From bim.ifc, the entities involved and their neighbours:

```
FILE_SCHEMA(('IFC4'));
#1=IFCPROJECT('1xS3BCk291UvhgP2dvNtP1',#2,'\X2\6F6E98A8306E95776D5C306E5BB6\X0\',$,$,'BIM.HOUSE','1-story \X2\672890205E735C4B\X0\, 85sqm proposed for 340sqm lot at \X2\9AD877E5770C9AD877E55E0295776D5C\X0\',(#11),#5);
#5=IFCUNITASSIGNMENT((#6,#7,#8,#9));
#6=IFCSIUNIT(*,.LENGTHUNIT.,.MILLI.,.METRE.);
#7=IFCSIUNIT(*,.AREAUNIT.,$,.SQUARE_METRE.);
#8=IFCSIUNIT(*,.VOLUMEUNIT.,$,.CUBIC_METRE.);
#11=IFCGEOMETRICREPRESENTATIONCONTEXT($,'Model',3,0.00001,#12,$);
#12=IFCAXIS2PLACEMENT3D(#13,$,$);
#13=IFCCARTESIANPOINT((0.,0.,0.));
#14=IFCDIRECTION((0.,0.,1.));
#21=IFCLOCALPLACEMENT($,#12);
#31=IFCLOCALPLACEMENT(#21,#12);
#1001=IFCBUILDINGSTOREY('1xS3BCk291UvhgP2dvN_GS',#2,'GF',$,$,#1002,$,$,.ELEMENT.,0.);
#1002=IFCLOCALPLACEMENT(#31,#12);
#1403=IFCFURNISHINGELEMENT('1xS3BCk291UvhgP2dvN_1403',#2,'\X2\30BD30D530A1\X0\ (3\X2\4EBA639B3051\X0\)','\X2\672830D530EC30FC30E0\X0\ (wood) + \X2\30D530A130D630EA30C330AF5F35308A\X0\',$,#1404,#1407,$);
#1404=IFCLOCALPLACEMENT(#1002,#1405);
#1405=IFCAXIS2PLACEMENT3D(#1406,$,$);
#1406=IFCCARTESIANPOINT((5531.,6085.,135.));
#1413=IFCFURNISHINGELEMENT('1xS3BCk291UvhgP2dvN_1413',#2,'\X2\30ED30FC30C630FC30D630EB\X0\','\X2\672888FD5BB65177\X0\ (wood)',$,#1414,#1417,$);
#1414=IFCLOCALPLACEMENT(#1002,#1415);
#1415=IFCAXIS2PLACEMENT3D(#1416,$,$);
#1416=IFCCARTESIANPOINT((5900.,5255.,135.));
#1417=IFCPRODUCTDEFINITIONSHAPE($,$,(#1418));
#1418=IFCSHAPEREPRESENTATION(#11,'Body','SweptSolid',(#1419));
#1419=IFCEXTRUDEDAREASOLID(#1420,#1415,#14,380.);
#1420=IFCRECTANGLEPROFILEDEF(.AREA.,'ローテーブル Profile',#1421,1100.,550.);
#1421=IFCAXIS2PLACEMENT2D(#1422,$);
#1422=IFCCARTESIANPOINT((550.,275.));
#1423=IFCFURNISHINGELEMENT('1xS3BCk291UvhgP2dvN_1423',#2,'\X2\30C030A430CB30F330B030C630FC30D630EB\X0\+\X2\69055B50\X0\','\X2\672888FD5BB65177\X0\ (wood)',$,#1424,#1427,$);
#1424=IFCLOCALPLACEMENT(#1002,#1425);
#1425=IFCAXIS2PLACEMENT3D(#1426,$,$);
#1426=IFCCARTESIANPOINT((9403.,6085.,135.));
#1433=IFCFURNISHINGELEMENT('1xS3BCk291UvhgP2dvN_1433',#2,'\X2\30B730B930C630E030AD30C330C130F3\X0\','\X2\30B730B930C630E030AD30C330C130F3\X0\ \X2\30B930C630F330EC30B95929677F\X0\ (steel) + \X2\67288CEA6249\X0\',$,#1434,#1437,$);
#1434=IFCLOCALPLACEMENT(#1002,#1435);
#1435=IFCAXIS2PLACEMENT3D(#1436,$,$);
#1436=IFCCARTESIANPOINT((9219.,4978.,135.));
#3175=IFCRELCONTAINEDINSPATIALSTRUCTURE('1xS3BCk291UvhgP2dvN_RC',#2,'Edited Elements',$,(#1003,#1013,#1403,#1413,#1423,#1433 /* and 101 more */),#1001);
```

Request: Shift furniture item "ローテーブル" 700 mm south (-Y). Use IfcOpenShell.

```python
import ifcopenshell
import ifcopenshell.api.geometry
import ifcopenshell.util.placement

model = ifcopenshell.open("bim.ifc")

item = model.by_guid("1xS3BCk291UvhgP2dvN_1413")
matrix = ifcopenshell.util.placement.get_local_placement(item.ObjectPlacement)
matrix[1, 3] -= 700.0
ifcopenshell.api.geometry.edit_object_placement(model, product=item, matrix=matrix, is_si=False)

print(ifcopenshell.util.placement.get_local_placement(item.ObjectPlacement).round(3) + 0.0)

model.write("bim-out.ifc")
```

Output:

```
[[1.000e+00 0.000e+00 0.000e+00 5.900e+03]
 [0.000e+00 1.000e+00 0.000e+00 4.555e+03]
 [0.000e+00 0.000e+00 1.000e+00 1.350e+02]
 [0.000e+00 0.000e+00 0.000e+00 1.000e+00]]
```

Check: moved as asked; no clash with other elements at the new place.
